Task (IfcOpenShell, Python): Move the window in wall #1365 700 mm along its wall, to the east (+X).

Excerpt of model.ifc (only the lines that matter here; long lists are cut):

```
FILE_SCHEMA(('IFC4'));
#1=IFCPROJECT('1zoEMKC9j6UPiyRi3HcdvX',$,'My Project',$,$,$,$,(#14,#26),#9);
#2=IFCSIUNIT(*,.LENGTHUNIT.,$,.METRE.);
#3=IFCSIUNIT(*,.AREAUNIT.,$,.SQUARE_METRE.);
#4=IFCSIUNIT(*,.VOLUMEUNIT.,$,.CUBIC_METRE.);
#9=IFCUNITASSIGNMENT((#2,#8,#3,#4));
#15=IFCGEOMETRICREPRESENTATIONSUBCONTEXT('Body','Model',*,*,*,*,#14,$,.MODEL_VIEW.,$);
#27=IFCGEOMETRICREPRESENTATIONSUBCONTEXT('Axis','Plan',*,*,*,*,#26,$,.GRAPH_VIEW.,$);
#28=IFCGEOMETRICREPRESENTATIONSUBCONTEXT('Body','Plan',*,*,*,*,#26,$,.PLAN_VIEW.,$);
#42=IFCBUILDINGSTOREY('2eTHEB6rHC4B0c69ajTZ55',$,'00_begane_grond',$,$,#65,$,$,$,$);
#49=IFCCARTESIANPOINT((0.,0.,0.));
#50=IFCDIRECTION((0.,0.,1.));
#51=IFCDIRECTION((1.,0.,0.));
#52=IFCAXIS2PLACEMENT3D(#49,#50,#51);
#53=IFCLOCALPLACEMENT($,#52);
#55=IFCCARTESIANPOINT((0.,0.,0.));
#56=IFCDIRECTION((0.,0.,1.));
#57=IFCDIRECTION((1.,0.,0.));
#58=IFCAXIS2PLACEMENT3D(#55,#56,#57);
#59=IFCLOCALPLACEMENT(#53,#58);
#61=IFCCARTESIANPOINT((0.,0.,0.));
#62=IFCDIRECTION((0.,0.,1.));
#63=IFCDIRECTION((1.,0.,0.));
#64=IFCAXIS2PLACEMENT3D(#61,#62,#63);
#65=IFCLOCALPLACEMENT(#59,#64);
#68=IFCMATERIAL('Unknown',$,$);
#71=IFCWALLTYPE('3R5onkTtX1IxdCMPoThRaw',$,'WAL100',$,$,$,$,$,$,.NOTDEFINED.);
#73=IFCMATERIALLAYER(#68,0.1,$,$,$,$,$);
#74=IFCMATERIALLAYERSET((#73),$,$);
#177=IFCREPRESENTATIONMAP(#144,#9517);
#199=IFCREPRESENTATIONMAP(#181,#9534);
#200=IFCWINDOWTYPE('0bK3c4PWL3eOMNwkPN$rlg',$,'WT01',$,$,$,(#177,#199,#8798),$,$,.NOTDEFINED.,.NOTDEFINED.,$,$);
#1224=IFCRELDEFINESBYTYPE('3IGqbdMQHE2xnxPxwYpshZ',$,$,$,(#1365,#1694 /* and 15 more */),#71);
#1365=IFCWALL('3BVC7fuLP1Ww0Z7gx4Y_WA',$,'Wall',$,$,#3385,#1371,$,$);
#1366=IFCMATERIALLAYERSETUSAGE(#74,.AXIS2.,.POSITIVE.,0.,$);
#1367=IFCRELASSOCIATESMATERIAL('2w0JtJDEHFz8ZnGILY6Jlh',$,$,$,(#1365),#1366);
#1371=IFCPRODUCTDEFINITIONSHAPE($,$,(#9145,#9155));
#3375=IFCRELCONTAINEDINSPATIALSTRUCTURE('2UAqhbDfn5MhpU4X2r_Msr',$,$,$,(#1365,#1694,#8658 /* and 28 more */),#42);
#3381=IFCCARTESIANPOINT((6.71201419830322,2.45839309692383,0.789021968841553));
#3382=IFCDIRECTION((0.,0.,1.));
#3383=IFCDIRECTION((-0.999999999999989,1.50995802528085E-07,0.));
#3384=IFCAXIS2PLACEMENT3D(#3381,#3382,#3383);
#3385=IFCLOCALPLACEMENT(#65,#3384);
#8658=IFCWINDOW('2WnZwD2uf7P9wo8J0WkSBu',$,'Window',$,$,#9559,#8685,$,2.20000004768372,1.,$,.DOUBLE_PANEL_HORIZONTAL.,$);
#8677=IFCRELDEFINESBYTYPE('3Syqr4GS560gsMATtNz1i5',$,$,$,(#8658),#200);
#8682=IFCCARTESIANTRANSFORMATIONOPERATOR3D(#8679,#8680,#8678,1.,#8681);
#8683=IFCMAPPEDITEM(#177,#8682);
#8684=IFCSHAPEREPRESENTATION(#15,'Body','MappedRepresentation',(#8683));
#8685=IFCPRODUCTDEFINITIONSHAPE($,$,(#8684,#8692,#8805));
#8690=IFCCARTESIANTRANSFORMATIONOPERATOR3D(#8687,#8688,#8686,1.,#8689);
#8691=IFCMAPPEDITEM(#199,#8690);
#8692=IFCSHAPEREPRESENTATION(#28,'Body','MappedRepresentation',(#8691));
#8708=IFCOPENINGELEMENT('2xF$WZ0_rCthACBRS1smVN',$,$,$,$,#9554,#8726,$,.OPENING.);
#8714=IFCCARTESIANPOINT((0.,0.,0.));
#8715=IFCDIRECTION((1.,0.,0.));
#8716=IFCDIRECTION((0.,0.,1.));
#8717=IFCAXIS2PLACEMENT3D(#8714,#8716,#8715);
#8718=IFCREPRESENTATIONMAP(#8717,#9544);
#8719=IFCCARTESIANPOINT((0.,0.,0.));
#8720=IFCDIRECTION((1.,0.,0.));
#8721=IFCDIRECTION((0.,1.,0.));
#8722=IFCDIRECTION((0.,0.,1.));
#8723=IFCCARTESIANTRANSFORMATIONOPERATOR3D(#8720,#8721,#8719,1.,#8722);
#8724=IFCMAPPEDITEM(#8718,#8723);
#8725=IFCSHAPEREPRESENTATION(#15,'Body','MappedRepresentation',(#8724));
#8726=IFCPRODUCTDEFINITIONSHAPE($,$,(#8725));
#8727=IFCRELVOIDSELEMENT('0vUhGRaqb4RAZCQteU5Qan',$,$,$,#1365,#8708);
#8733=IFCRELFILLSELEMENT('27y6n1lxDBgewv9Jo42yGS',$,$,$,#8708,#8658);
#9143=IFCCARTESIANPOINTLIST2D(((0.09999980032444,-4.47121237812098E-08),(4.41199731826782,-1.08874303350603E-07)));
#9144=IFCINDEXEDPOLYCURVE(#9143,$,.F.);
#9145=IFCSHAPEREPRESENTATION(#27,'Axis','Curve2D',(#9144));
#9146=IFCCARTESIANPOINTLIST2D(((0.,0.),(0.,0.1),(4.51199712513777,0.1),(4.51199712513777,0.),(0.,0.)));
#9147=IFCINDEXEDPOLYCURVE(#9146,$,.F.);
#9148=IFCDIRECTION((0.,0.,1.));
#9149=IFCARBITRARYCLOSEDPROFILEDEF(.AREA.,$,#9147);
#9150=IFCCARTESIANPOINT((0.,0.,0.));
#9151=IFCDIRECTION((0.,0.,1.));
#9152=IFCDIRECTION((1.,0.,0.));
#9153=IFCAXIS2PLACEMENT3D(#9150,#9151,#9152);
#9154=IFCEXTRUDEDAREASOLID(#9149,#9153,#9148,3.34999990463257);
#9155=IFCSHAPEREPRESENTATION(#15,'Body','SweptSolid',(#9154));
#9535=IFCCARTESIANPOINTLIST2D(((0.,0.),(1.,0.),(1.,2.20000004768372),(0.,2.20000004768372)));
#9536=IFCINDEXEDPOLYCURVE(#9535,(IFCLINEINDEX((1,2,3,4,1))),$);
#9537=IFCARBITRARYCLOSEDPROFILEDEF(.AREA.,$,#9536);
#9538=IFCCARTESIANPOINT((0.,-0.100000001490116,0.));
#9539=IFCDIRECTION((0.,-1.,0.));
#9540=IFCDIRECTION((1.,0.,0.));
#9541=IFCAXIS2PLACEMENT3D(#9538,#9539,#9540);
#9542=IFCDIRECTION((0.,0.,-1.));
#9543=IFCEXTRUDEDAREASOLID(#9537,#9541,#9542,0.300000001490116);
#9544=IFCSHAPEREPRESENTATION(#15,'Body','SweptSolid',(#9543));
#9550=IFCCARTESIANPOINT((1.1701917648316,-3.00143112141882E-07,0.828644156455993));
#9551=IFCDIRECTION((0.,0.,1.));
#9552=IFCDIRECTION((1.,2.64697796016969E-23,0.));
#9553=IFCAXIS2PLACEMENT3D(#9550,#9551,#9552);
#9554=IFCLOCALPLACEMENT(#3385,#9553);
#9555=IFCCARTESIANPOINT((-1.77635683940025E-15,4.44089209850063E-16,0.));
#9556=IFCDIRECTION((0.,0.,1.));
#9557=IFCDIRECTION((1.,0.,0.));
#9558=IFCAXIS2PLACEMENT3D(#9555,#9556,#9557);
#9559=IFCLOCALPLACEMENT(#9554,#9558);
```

```python
import ifcopenshell
import ifcopenshell.api.geometry
import ifcopenshell.util.placement
import ifcopenshell.util.unit

model = ifcopenshell.open("model.ifc")
unit_scale = ifcopenshell.util.unit.calculate_unit_scale(model)

window = model.by_guid("2WnZwD2uf7P9wo8J0WkSBu")
opening = window.FillsVoids[0].RelatingOpeningElement
wall = opening.VoidsElements[0].RelatingBuildingElement

wall_matrix = ifcopenshell.util.placement.get_local_placement(wall.ObjectPlacement)
shift = wall_matrix[:3, 0] * -0.7 / unit_scale
before = ifcopenshell.util.placement.get_local_placement(window.ObjectPlacement)[:3, 3].copy()

# The window is placed relative to its opening, so it follows when the opening moves.
matrix = ifcopenshell.util.placement.get_local_placement(opening.ObjectPlacement)
matrix[:3, 3] += shift
ifcopenshell.api.geometry.edit_object_placement(
    model, product=opening, matrix=matrix, is_si=False, should_transform_children=True
)

after = ifcopenshell.util.placement.get_local_placement(window.ObjectPlacement)[:3, 3]
print("window moved by", (after - before).round(3) + 0.0)

model.write("model-out.ifc")
```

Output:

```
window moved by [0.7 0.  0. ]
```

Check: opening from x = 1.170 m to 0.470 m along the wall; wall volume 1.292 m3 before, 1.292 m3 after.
